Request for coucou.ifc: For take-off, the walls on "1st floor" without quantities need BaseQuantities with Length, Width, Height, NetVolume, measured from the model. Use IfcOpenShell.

First a look at what the model holds.

```python
import ifcopenshell
import ifcopenshell.util.element
import ifcopenshell.util.unit

model = ifcopenshell.open("coucou.ifc")
print(model.schema)
for unit_type in ("LENGTHUNIT", "AREAUNIT", "VOLUMEUNIT"):
    print(unit_type, ifcopenshell.util.unit.calculate_unit_scale(model, unit_type))
storey = next(s for s in model.by_type("IfcBuildingStorey") if s.Name == "1st floor")
walls = [e for e in ifcopenshell.util.element.get_decomposition(storey) if e.is_a("IfcWall")]
for e in sorted(walls, key=lambda e: e.id()):
    print(e.id(), e.is_a(), e.Name, list(ifcopenshell.util.element.get_psets(e, qtos_only=True)), sep=" | ")
```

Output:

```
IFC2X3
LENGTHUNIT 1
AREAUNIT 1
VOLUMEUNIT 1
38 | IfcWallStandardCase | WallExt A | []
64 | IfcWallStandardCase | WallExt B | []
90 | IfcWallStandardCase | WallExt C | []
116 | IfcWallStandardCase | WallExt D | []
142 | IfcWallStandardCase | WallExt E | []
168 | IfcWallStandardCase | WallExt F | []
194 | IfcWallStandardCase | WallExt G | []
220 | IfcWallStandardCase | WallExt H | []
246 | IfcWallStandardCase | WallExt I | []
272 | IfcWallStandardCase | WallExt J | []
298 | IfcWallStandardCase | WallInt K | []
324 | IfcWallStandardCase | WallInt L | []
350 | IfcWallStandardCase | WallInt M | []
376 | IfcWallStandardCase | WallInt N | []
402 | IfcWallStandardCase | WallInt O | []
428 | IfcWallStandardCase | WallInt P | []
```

```python
import ifcopenshell
import ifcopenshell.api.pset
import ifcopenshell.geom
import ifcopenshell.util.element
import ifcopenshell.util.shape
import ifcopenshell.util.unit

model = ifcopenshell.open("coucou.ifc")
unit_scale = ifcopenshell.util.unit.calculate_unit_scale(model)
volume_scale = ifcopenshell.util.unit.calculate_unit_scale(model, "VOLUMEUNIT")
settings = ifcopenshell.geom.settings()

storey = next(s for s in model.by_type("IfcBuildingStorey") if s.Name == "1st floor")
walls = [e for e in ifcopenshell.util.element.get_decomposition(storey) if e.is_a("IfcWall")]

for e in sorted(walls, key=lambda e: e.id()):
    if ifcopenshell.util.element.get_psets(e, qtos_only=True, should_inherit=False):
        continue
    # Geometry comes back in metres, in the element's own axes.
    shape = ifcopenshell.geom.create_shape(settings, e)
    values = {
        "Length": ifcopenshell.util.shape.get_x(shape.geometry) / unit_scale,
        "Width": ifcopenshell.util.shape.get_y(shape.geometry) / unit_scale,
        "Height": ifcopenshell.util.shape.get_z(shape.geometry) / unit_scale,
        "NetVolume": ifcopenshell.util.shape.get_volume(shape.geometry) / volume_scale,
    }
    qto = ifcopenshell.api.pset.add_qto(model, product=e, name="BaseQuantities")
    ifcopenshell.api.pset.edit_qto(model, qto=qto, properties=values)
    print(e.id(), {k: round(v, 3) for k, v in values.items()})

model.write("coucou_edited.ifc")
```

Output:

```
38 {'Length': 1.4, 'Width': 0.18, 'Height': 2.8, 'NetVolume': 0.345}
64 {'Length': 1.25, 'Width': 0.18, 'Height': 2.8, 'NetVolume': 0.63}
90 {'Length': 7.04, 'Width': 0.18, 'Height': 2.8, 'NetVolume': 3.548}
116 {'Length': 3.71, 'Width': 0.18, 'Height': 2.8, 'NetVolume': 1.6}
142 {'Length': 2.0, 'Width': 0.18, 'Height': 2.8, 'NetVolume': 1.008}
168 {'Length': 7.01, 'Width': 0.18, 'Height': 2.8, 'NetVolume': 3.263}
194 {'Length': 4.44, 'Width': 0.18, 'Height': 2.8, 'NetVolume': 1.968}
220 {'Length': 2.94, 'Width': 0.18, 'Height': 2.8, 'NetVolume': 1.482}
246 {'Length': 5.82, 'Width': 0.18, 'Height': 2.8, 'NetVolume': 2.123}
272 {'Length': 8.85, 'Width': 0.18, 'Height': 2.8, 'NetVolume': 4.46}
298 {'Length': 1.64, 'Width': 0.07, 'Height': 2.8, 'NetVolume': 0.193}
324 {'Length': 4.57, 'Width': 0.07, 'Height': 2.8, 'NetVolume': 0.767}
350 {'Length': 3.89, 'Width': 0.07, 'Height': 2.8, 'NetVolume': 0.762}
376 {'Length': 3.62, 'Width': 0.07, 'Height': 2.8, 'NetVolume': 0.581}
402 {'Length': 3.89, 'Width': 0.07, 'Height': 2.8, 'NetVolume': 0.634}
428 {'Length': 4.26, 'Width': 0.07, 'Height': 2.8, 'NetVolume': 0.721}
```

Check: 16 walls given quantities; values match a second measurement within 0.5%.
